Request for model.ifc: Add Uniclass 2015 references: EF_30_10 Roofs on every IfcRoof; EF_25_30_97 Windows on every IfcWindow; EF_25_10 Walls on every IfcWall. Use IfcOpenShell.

First a look at what the model holds.

```python
import ifcopenshell

model = ifcopenshell.open("model.ifc")
print(model.schema)
print("classifications:", [c.Name for c in model.by_type("IfcClassification")])
for ifc_class in ("IfcDoor", "IfcRoof", "IfcStair", "IfcWall", "IfcWindow"):
    print(ifc_class, len(model.by_type(ifc_class)))
```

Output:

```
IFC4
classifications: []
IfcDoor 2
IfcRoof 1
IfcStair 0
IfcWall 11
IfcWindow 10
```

```python
import ifcopenshell
import ifcopenshell.api.classification

model = ifcopenshell.open("model.ifc")

system = ifcopenshell.api.classification.add_classification(model, classification="Uniclass 2015")

codes = {
    "IfcRoof": ("EF_30_10", "Roofs"),
    "IfcWindow": ("EF_25_30_97", "Windows"),
    "IfcWall": ("EF_25_10", "Walls"),
}
for ifc_class, (code, name) in codes.items():
    products = model.by_type(ifc_class)
    ifcopenshell.api.classification.add_reference(
        model, products=products, classification=system, identification=code, name=name
    )
    print(code, len(products))

model.write("model_v2.ifc")
```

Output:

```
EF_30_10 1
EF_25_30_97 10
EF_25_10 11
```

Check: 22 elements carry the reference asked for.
